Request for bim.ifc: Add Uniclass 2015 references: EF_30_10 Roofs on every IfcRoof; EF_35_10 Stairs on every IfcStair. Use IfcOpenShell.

First a look at what the model holds.

```python
import ifcopenshell

model = ifcopenshell.open("bim.ifc")
print(model.schema)
print("classifications:", [c.Name for c in model.by_type("IfcClassification")])
for ifc_class in ("IfcDoor", "IfcRoof", "IfcStair", "IfcWall", "IfcWindow"):
    print(ifc_class, len(model.by_type(ifc_class)))
```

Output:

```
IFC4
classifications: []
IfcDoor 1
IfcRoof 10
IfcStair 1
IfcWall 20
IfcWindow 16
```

```python
import ifcopenshell
import ifcopenshell.api.classification

model = ifcopenshell.open("bim.ifc")

system = ifcopenshell.api.classification.add_classification(model, classification="Uniclass 2015")

codes = {
    "IfcRoof": ("EF_30_10", "Roofs"),
    "IfcStair": ("EF_35_10", "Stairs"),
}
for ifc_class, (code, name) in codes.items():
    products = model.by_type(ifc_class)
    ifcopenshell.api.classification.add_reference(
        model, products=products, classification=system, identification=code, name=name
    )
    print(code, len(products))

model.write("bim_updated.ifc")
```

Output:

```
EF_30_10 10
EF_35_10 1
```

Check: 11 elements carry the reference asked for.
